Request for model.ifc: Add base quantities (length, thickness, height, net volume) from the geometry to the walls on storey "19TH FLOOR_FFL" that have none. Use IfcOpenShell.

First a look at what the model holds.

```python
import ifcopenshell
import ifcopenshell.util.element
import ifcopenshell.util.unit

model = ifcopenshell.open("model.ifc")
print(model.schema)
for unit_type in ("LENGTHUNIT", "AREAUNIT", "VOLUMEUNIT"):
    print(unit_type, ifcopenshell.util.unit.calculate_unit_scale(model, unit_type))
storey = next(s for s in model.by_type("IfcBuildingStorey") if s.Name == "19TH FLOOR_FFL")
walls = [e for e in ifcopenshell.util.element.get_decomposition(storey) if e.is_a("IfcWall")]
for e in sorted(walls, key=lambda e: e.id()):
    print(e.id(), e.is_a(), e.Name, list(ifcopenshell.util.element.get_psets(e, qtos_only=True)), sep=" | ")
```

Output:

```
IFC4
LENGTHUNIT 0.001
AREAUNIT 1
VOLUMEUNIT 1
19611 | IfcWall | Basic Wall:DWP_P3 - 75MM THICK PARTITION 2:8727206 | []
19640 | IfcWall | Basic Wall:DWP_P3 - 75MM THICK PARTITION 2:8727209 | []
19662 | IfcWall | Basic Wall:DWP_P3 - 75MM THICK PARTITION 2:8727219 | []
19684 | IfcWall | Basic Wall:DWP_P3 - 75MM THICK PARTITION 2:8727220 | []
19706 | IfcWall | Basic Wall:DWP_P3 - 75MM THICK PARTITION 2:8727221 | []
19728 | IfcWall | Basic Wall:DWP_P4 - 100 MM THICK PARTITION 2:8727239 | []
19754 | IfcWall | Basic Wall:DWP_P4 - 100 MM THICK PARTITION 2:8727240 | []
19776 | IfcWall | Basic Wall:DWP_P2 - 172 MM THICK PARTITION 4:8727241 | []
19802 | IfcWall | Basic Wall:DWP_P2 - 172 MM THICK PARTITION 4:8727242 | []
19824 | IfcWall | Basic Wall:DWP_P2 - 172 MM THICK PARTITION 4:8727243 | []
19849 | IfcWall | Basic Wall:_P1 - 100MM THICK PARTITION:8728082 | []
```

```python
import ifcopenshell
import ifcopenshell.api.pset
import ifcopenshell.geom
import ifcopenshell.util.element
import ifcopenshell.util.shape
import ifcopenshell.util.unit

model = ifcopenshell.open("model.ifc")
unit_scale = ifcopenshell.util.unit.calculate_unit_scale(model)
volume_scale = ifcopenshell.util.unit.calculate_unit_scale(model, "VOLUMEUNIT")
settings = ifcopenshell.geom.settings()

storey = next(s for s in model.by_type("IfcBuildingStorey") if s.Name == "19TH FLOOR_FFL")
walls = [e for e in ifcopenshell.util.element.get_decomposition(storey) if e.is_a("IfcWall")]

for e in sorted(walls, key=lambda e: e.id()):
    if ifcopenshell.util.element.get_psets(e, qtos_only=True, should_inherit=False):
        continue
    # Geometry comes back in metres, in the element's own axes.
    shape = ifcopenshell.geom.create_shape(settings, e)
    values = {
        "Length": ifcopenshell.util.shape.get_x(shape.geometry) / unit_scale,
        "Width": ifcopenshell.util.shape.get_y(shape.geometry) / unit_scale,
        "Height": ifcopenshell.util.shape.get_z(shape.geometry) / unit_scale,
        "NetVolume": ifcopenshell.util.shape.get_volume(shape.geometry) / volume_scale,
    }
    qto = ifcopenshell.api.pset.add_qto(model, product=e, name="Qto_WallBaseQuantities")
    ifcopenshell.api.pset.edit_qto(model, qto=qto, properties=values)
    print(e.id(), {k: round(v, 3) for k, v in values.items()})

model.write("model_rev.ifc")
```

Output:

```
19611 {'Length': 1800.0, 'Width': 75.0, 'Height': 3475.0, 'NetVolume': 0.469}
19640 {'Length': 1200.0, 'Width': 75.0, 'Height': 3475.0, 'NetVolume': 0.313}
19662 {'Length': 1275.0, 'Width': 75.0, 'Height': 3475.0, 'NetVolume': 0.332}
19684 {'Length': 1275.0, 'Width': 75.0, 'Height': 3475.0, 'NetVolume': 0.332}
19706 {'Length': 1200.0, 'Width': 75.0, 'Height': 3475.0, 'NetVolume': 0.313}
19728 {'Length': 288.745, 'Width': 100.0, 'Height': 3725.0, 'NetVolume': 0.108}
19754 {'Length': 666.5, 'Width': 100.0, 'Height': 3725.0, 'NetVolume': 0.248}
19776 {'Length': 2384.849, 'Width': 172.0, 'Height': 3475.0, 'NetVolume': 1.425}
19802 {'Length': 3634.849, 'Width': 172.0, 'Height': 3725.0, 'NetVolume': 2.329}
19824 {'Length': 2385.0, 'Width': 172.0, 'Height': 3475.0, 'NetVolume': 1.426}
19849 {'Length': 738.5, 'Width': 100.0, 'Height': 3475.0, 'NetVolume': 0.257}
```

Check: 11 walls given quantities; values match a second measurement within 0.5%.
